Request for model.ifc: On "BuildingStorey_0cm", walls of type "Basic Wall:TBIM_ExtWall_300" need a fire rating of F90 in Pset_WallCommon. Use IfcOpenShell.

First a look at what the model holds.

```python
import ifcopenshell
import ifcopenshell.util.element

model = ifcopenshell.open("model.ifc")
print(model.schema)
storey = next(s for s in model.by_type("IfcBuildingStorey") if s.Name == "BuildingStorey_0cm")
walls = [e for e in ifcopenshell.util.element.get_decomposition(storey) if e.is_a("IfcWall")]
seen = {}
for e in walls:
    element_type = ifcopenshell.util.element.get_type(e)
    key = (element_type.Name if element_type != e and element_type else None, ifcopenshell.util.element.get_pset(e, "Pset_WallCommon", "FireRating"))
    seen[key] = seen.get(key, 0) + 1
for (name, value), count in sorted(seen.items(), key=str):
    print(count, "x", name, "|", value)
```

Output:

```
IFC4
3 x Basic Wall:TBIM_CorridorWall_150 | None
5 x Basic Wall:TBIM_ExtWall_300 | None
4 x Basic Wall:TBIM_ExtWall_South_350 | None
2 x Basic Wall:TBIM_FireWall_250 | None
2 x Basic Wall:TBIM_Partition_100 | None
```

```python
import ifcopenshell
import ifcopenshell.api.pset
import ifcopenshell.util.element

model = ifcopenshell.open("model.ifc")

storey = next(s for s in model.by_type("IfcBuildingStorey") if s.Name == "BuildingStorey_0cm")
walls = [e for e in ifcopenshell.util.element.get_decomposition(storey) if e.is_a("IfcWall")]

count = 0
for e in walls:
    element_type = ifcopenshell.util.element.get_type(e)
    if element_type in (None, e) or element_type.Name != "Basic Wall:TBIM_ExtWall_300":
        continue
    # add_pset returns the element's existing set when there is one.
    pset = ifcopenshell.api.pset.add_pset(model, product=e, name="Pset_WallCommon")
    ifcopenshell.api.pset.edit_pset(model, pset=pset, properties={"FireRating": "F90"})
    count += 1

print(count, "walls updated")

model.write("model_updated.ifc")
```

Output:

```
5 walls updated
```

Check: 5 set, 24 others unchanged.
